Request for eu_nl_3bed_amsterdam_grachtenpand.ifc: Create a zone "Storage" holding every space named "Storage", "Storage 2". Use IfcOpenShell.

First a look at what the model holds.

```python
import ifcopenshell

model = ifcopenshell.open("eu_nl_3bed_amsterdam_grachtenpand.ifc")
print(model.schema)
seen = {}
for space in model.by_type("IfcSpace"):
    seen[space.LongName] = seen.get(space.LongName, 0) + 1
for name, count in sorted(seen.items(), key=str):
    print(count, "x", name)
print("zones:", [z.Name for z in model.by_type("IfcZone")][:20])
```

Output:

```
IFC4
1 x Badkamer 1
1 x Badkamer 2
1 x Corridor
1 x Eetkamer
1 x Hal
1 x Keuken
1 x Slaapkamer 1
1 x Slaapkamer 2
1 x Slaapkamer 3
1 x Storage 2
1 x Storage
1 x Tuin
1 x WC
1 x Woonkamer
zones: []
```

```python
import ifcopenshell
import ifcopenshell.api.group
import ifcopenshell.api.root

model = ifcopenshell.open("eu_nl_3bed_amsterdam_grachtenpand.ifc")

names = {"Storage", "Storage 2"}
spaces = [s for s in model.by_type("IfcSpace") if s.LongName in names]

zone = ifcopenshell.api.root.create_entity(model, ifc_class="IfcZone", name="Storage")
ifcopenshell.api.group.assign_group(model, products=spaces, group=zone)
print(len(spaces), "spaces in", zone.Name)

model.write("eu_nl_3bed_amsterdam_grachtenpand_edited.ifc")
```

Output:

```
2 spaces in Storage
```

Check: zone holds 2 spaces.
